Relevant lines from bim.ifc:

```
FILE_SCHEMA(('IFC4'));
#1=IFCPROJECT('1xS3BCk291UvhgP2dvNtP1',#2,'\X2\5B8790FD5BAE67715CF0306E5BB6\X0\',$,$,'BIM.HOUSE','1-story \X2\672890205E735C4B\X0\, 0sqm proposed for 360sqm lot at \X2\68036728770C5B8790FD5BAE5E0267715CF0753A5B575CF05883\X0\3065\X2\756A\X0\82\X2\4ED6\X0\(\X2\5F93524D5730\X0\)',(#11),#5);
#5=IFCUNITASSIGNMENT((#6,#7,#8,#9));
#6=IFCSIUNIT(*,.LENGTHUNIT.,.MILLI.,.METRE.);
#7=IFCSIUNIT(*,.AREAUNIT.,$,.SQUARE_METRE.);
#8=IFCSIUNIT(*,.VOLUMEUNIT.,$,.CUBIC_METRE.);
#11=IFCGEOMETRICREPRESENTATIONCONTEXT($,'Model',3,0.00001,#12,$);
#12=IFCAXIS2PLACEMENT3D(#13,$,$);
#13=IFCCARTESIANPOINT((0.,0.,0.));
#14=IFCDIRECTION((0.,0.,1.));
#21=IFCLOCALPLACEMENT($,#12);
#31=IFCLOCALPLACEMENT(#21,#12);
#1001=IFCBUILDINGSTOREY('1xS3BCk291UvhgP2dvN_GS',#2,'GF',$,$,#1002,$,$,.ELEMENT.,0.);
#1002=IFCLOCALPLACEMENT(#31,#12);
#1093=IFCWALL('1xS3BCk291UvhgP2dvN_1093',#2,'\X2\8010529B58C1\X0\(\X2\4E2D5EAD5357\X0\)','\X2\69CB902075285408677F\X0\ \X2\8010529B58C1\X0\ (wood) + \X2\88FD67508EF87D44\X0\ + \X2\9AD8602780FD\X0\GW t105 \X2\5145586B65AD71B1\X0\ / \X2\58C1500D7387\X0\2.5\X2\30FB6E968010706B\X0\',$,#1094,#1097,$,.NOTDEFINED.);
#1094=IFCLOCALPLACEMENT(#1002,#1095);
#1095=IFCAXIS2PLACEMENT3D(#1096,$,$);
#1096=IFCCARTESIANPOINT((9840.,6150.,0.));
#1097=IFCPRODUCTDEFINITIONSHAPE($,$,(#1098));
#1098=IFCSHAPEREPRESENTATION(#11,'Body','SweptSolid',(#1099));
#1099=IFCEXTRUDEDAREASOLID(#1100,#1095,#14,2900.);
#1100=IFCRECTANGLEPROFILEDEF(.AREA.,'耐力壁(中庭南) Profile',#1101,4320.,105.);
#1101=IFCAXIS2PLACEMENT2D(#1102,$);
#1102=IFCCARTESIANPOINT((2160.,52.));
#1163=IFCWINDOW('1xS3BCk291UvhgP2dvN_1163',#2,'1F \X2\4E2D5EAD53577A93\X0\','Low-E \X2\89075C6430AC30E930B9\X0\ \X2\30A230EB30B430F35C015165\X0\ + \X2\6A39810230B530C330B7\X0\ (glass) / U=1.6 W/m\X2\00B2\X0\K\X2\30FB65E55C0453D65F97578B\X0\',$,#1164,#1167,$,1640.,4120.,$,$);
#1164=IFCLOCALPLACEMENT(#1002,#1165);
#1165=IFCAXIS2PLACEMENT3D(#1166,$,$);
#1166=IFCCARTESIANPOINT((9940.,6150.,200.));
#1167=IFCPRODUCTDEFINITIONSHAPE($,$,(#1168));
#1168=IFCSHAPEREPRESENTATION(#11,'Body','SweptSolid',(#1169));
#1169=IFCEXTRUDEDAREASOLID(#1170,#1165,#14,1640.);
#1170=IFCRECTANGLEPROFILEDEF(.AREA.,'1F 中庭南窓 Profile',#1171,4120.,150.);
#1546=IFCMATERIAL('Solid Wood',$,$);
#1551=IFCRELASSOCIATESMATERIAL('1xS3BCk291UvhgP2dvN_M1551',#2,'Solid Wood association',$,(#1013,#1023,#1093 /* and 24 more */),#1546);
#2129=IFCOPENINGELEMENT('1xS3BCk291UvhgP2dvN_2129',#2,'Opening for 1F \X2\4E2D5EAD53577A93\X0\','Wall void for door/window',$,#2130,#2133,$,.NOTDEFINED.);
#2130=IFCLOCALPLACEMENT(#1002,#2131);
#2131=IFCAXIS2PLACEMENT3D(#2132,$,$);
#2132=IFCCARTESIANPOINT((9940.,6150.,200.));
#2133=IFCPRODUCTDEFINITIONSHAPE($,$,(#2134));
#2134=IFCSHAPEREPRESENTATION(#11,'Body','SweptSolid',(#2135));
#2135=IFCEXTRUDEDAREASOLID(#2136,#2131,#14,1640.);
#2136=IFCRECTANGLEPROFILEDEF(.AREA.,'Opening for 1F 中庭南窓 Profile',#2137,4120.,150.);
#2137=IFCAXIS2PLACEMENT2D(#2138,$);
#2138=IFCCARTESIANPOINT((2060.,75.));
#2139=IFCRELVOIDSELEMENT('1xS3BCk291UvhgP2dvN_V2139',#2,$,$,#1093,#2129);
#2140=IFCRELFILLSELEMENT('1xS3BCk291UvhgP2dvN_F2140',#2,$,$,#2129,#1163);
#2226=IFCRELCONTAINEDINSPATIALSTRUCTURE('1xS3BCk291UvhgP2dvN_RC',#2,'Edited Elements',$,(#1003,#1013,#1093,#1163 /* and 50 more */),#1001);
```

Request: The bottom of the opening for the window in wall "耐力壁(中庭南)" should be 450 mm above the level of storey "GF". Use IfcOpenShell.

```python
import numpy as np
import ifcopenshell
import ifcopenshell.api.geometry
import ifcopenshell.geom
import ifcopenshell.util.element
import ifcopenshell.util.placement
import ifcopenshell.util.shape
import ifcopenshell.util.unit

model = ifcopenshell.open("bim.ifc")
unit_scale = ifcopenshell.util.unit.calculate_unit_scale(model)

window = model.by_id(1163)
opening = window.FillsVoids[0].RelatingOpeningElement
storey = ifcopenshell.util.element.get_container(window, ifc_class="IfcBuildingStorey")
level = ifcopenshell.util.placement.get_local_placement(storey.ObjectPlacement)[2, 3]

# The opening's origin need not be at the sill, so measure its lowest point.
shape = ifcopenshell.geom.create_shape(ifcopenshell.geom.settings(), opening)
bottom = ifcopenshell.util.shape.get_shape_bottom_elevation(shape, shape.geometry) / unit_scale
dz = level + 450.0 - bottom

shift = np.array([0.0, 0.0, dz])
# The window is not placed relative to its opening, so move both.
for product in (opening, window):
    matrix = ifcopenshell.util.placement.get_local_placement(product.ObjectPlacement)
    matrix[:3, 3] += shift
    ifcopenshell.api.geometry.edit_object_placement(model, product=product, matrix=matrix, is_si=False)

print(f"moved by {dz * unit_scale:+.3f} m")

model.write("bim_rev.ifc")
```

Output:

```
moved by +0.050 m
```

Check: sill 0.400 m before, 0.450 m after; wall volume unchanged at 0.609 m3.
